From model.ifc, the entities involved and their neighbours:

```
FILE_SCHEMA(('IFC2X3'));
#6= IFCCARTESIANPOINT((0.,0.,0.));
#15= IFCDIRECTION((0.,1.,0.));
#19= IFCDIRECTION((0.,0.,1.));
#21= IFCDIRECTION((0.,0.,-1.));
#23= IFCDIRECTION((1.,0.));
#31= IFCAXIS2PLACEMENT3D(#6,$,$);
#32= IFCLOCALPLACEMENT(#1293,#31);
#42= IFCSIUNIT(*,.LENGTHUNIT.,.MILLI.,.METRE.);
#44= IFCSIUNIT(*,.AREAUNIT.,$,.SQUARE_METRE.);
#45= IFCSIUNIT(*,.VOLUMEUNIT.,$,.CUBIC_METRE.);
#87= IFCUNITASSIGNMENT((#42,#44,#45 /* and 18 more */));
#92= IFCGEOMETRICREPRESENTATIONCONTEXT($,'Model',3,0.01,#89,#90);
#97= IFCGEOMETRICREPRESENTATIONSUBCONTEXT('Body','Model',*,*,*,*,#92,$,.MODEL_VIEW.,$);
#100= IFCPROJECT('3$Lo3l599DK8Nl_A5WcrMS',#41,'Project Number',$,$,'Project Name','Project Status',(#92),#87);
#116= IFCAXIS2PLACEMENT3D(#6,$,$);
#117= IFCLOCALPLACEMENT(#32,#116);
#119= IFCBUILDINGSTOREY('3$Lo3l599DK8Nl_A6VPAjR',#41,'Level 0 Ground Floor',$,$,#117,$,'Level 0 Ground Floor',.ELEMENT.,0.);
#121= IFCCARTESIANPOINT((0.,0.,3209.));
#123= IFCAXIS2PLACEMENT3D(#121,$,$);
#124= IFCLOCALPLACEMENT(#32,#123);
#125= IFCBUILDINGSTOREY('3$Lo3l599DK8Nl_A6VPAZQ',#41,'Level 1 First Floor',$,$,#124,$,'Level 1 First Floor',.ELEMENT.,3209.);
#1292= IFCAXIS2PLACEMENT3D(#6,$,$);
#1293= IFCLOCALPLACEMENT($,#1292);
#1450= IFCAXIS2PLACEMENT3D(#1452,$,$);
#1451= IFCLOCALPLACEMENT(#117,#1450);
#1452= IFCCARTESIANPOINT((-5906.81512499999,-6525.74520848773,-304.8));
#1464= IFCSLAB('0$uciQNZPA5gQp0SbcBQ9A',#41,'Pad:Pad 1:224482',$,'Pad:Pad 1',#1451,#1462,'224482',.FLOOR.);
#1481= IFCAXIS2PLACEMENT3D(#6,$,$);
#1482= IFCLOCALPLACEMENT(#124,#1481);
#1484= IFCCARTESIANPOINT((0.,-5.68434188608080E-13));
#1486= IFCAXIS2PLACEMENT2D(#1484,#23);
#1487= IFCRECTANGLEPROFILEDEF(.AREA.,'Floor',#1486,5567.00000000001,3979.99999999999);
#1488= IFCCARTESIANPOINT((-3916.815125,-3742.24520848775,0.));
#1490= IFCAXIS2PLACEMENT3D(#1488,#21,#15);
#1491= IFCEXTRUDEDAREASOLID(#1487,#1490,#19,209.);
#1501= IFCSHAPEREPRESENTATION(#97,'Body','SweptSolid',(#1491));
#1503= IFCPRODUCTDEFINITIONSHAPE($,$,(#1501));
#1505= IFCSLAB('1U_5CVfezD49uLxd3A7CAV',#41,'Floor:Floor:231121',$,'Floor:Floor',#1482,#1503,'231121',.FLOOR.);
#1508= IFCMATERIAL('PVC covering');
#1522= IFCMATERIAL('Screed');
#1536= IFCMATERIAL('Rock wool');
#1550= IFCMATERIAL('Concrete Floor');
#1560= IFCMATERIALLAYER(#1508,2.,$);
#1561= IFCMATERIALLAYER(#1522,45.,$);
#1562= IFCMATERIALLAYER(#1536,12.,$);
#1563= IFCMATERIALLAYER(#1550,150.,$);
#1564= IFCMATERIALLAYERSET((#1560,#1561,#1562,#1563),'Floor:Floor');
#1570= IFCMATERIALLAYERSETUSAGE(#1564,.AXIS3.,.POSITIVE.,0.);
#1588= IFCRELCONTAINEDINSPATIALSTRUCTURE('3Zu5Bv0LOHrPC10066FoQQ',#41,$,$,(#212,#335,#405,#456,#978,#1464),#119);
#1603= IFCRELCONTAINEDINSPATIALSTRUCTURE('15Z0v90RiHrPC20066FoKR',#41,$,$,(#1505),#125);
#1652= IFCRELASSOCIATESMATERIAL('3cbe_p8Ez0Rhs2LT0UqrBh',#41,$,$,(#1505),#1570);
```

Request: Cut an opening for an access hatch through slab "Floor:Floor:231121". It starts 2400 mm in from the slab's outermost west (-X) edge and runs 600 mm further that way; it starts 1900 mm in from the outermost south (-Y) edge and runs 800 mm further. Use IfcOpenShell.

```python
import numpy as np
import ifcopenshell
import ifcopenshell.api.feature
import ifcopenshell.api.geometry
import ifcopenshell.api.root
import ifcopenshell.geom
import ifcopenshell.util.placement
import ifcopenshell.util.representation
import ifcopenshell.util.shape
import ifcopenshell.util.unit

model = ifcopenshell.open("model.ifc")
unit_scale = ifcopenshell.util.unit.calculate_unit_scale(model)
settings = ifcopenshell.geom.settings()


def volume(element):
    """Net volume in cubic metres, openings subtracted."""
    shape = ifcopenshell.geom.create_shape(settings, element)
    return ifcopenshell.util.shape.get_volume(shape.geometry)


slab = model.by_id(1505)
before = volume(slab)

# Extent in the slab's own axes, in metres. The edges named are its -X and -Y sides.
slab_shape = ifcopenshell.geom.create_shape(settings, slab)
vertices = ifcopenshell.util.shape.get_vertices(slab_shape.geometry)
x_min, y_min, bottom = vertices.min(axis=0)
top = vertices[:, 2].max()

opening = ifcopenshell.api.root.create_entity(model, ifc_class="IfcOpeningElement", name="Access hatch opening")
context = ifcopenshell.util.representation.get_context(model, "Model", "Body", "MODEL_VIEW")
width, depth = 0.6, 0.8
outline = [(0.0, 0.0), (width, 0.0), (width, depth), (0.0, depth), (0.0, 0.0)]
# Overshoot both faces by 50 mm so the cut is clean.
shape = ifcopenshell.api.geometry.add_slab_representation(
    model, context=context, depth=top - bottom + 0.1, polyline=outline
)
ifcopenshell.api.geometry.assign_representation(model, product=opening, representation=shape)

matrix = ifcopenshell.util.placement.get_local_placement(slab.ObjectPlacement)
matrix[:, 3] = matrix @ np.append(np.array([x_min + 2.4, y_min + 1.9, bottom - 0.05]) / unit_scale, 1.0)
ifcopenshell.api.geometry.edit_object_placement(model, product=opening, matrix=matrix, is_si=False)
ifcopenshell.api.feature.add_feature(model, feature=opening, element=slab)

after = volume(slab)

print(f"slab volume {before:.3f} -> {after:.3f} m3")

model.write("model_updated.ifc")
```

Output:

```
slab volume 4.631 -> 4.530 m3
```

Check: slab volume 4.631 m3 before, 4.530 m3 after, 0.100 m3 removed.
